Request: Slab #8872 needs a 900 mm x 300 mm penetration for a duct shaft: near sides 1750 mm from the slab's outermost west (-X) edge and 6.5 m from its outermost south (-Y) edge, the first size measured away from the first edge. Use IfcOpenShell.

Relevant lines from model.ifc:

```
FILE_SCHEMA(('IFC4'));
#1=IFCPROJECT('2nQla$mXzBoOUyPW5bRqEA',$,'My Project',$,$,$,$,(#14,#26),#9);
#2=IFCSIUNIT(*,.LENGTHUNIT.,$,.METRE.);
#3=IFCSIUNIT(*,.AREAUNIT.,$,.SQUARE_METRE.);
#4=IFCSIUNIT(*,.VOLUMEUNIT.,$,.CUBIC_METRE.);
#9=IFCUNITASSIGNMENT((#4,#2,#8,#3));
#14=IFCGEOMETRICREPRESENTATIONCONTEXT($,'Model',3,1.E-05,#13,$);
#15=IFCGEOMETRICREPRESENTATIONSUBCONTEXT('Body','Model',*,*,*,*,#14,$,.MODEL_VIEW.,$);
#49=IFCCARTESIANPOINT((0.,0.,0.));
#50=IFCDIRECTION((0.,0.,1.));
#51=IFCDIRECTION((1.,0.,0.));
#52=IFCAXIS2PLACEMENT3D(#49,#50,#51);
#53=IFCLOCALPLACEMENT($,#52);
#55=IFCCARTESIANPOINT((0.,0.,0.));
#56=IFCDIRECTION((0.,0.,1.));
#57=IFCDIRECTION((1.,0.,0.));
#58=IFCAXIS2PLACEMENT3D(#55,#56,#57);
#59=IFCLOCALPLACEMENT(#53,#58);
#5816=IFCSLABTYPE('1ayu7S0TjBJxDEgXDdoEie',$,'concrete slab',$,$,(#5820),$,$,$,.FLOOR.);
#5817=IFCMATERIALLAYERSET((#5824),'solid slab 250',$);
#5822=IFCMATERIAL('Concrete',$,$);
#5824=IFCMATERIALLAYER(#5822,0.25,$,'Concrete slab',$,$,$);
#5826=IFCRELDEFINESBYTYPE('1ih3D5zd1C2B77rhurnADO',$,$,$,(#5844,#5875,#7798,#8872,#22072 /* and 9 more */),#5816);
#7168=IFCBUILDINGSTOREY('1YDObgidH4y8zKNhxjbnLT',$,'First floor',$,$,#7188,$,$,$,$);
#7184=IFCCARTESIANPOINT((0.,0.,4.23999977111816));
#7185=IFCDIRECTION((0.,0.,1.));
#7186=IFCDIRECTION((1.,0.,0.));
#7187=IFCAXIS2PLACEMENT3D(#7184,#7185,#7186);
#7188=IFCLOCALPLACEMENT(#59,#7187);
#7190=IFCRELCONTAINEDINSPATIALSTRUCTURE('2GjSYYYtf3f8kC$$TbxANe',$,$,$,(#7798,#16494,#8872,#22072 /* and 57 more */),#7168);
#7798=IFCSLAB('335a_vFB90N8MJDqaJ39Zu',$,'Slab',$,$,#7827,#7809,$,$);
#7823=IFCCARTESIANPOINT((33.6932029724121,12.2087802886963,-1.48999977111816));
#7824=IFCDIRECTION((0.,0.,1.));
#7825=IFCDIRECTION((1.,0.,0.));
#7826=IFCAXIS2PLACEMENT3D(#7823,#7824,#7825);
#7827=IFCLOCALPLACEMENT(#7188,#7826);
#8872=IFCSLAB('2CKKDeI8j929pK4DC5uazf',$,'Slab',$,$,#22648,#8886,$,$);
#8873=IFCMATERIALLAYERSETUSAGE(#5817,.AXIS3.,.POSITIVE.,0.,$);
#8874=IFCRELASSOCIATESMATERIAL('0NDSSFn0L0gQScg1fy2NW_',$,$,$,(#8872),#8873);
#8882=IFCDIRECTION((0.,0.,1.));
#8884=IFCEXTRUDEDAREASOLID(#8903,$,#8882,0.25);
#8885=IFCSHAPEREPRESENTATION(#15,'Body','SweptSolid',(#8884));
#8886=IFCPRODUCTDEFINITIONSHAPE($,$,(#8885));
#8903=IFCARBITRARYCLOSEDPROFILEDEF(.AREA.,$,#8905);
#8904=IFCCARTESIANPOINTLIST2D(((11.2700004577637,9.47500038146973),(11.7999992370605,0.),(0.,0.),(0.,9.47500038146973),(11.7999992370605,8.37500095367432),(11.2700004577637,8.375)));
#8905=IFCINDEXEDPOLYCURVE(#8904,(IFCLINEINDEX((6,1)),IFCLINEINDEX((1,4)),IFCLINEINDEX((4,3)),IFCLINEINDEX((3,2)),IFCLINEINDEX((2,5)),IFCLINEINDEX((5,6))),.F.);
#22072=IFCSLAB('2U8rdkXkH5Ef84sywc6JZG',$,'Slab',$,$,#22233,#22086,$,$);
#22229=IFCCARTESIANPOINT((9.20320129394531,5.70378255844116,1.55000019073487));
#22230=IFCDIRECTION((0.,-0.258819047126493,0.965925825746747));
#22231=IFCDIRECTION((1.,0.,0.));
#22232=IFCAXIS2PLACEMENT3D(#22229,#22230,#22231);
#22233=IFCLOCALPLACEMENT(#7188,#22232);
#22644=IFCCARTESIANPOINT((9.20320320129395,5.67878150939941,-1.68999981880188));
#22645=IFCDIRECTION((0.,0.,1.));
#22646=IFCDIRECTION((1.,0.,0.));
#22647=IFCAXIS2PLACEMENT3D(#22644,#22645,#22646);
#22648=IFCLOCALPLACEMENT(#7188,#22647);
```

```python
import numpy as np
import ifcopenshell
import ifcopenshell.api.feature
import ifcopenshell.api.geometry
import ifcopenshell.api.root
import ifcopenshell.geom
import ifcopenshell.util.placement
import ifcopenshell.util.representation
import ifcopenshell.util.shape
import ifcopenshell.util.unit

model = ifcopenshell.open("model.ifc")
unit_scale = ifcopenshell.util.unit.calculate_unit_scale(model)
settings = ifcopenshell.geom.settings()


def volume(element):
    """Net volume in cubic metres, openings subtracted."""
    shape = ifcopenshell.geom.create_shape(settings, element)
    return ifcopenshell.util.shape.get_volume(shape.geometry)


slab = model.by_guid("2CKKDeI8j929pK4DC5uazf")
before = volume(slab)

# Extent in the slab's own axes, in metres. The edges named are its -X and -Y sides.
slab_shape = ifcopenshell.geom.create_shape(settings, slab)
vertices = ifcopenshell.util.shape.get_vertices(slab_shape.geometry)
x_min, y_min, bottom = vertices.min(axis=0)
top = vertices[:, 2].max()

opening = ifcopenshell.api.root.create_entity(model, ifc_class="IfcOpeningElement", name="Duct shaft opening", predefined_type="OPENING")
context = ifcopenshell.util.representation.get_context(model, "Model", "Body", "MODEL_VIEW")
width, depth = 0.9, 0.3
outline = [(0.0, 0.0), (width, 0.0), (width, depth), (0.0, depth), (0.0, 0.0)]
# Overshoot both faces by 50 mm so the cut is clean.
shape = ifcopenshell.api.geometry.add_slab_representation(
    model, context=context, depth=top - bottom + 0.1, polyline=outline
)
ifcopenshell.api.geometry.assign_representation(model, product=opening, representation=shape)

matrix = ifcopenshell.util.placement.get_local_placement(slab.ObjectPlacement)
matrix[:, 3] = matrix @ np.append(np.array([x_min + 1.75, y_min + 6.5, bottom - 0.05]) / unit_scale, 1.0)
ifcopenshell.api.geometry.edit_object_placement(model, product=opening, matrix=matrix, is_si=False)
ifcopenshell.api.feature.add_feature(model, feature=opening, element=slab)

after = volume(slab)

print(f"slab volume {before:.3f} -> {after:.3f} m3")

model.write("model-out.ifc")
```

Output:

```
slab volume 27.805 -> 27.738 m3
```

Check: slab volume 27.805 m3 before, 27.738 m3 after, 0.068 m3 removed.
